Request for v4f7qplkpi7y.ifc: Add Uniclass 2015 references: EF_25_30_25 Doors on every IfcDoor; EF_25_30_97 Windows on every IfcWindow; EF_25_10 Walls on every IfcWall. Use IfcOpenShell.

First a look at what the model holds.

```python
import ifcopenshell

model = ifcopenshell.open("v4f7qplkpi7y.ifc")
print(model.schema)
print("classifications:", [c.Name for c in model.by_type("IfcClassification")])
for ifc_class in ("IfcDoor", "IfcRoof", "IfcStair", "IfcWall", "IfcWindow"):
    print(ifc_class, len(model.by_type(ifc_class)))
```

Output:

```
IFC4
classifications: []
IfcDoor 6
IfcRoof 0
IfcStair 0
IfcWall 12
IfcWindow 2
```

```python
import ifcopenshell
import ifcopenshell.api.classification

model = ifcopenshell.open("v4f7qplkpi7y.ifc")

system = ifcopenshell.api.classification.add_classification(model, classification="Uniclass 2015")

codes = {
    "IfcDoor": ("EF_25_30_25", "Doors"),
    "IfcWindow": ("EF_25_30_97", "Windows"),
    "IfcWall": ("EF_25_10", "Walls"),
}
for ifc_class, (code, name) in codes.items():
    products = model.by_type(ifc_class)
    ifcopenshell.api.classification.add_reference(
        model, products=products, classification=system, identification=code, name=name
    )
    print(code, len(products))

model.write("v4f7qplkpi7y_v2.ifc")
```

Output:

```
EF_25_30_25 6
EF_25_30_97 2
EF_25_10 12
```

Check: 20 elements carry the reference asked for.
